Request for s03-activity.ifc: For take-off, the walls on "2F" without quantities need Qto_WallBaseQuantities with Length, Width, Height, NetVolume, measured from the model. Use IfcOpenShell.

First a look at what the model holds.

```python
import ifcopenshell
import ifcopenshell.util.element
import ifcopenshell.util.unit

model = ifcopenshell.open("s03-activity.ifc")
print(model.schema)
for unit_type in ("LENGTHUNIT", "AREAUNIT", "VOLUMEUNIT"):
    print(unit_type, ifcopenshell.util.unit.calculate_unit_scale(model, unit_type))
storey = next(s for s in model.by_type("IfcBuildingStorey") if s.Name == "2F")
walls = [e for e in ifcopenshell.util.element.get_decomposition(storey) if e.is_a("IfcWall")]
for e in sorted(walls, key=lambda e: e.id()):
    print(e.id(), e.is_a(), e.Name, list(ifcopenshell.util.element.get_psets(e, qtos_only=True)), sep=" | ")
```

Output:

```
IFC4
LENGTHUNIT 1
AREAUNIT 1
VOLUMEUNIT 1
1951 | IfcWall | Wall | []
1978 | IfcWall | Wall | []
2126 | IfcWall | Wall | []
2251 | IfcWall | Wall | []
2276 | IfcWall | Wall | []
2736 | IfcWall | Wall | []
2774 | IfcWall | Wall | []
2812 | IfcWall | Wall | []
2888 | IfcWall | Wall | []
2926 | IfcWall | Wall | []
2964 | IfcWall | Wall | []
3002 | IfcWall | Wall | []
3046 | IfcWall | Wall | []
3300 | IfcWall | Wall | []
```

```python
import ifcopenshell
import ifcopenshell.api.pset
import ifcopenshell.geom
import ifcopenshell.util.element
import ifcopenshell.util.shape
import ifcopenshell.util.unit

model = ifcopenshell.open("s03-activity.ifc")
unit_scale = ifcopenshell.util.unit.calculate_unit_scale(model)
volume_scale = ifcopenshell.util.unit.calculate_unit_scale(model, "VOLUMEUNIT")
settings = ifcopenshell.geom.settings()

storey = next(s for s in model.by_type("IfcBuildingStorey") if s.Name == "2F")
walls = [e for e in ifcopenshell.util.element.get_decomposition(storey) if e.is_a("IfcWall")]

for e in sorted(walls, key=lambda e: e.id()):
    if ifcopenshell.util.element.get_psets(e, qtos_only=True, should_inherit=False):
        continue
    # Geometry comes back in metres, in the element's own axes.
    shape = ifcopenshell.geom.create_shape(settings, e)
    values = {
        "Length": ifcopenshell.util.shape.get_x(shape.geometry) / unit_scale,
        "Width": ifcopenshell.util.shape.get_y(shape.geometry) / unit_scale,
        "Height": ifcopenshell.util.shape.get_z(shape.geometry) / unit_scale,
        "NetVolume": ifcopenshell.util.shape.get_volume(shape.geometry) / volume_scale,
    }
    qto = ifcopenshell.api.pset.add_qto(model, product=e, name="Qto_WallBaseQuantities")
    ifcopenshell.api.pset.edit_qto(model, qto=qto, properties=values)
    print(e.id(), {k: round(v, 3) for k, v in values.items()})

model.write("s03-activity_v2.ifc")
```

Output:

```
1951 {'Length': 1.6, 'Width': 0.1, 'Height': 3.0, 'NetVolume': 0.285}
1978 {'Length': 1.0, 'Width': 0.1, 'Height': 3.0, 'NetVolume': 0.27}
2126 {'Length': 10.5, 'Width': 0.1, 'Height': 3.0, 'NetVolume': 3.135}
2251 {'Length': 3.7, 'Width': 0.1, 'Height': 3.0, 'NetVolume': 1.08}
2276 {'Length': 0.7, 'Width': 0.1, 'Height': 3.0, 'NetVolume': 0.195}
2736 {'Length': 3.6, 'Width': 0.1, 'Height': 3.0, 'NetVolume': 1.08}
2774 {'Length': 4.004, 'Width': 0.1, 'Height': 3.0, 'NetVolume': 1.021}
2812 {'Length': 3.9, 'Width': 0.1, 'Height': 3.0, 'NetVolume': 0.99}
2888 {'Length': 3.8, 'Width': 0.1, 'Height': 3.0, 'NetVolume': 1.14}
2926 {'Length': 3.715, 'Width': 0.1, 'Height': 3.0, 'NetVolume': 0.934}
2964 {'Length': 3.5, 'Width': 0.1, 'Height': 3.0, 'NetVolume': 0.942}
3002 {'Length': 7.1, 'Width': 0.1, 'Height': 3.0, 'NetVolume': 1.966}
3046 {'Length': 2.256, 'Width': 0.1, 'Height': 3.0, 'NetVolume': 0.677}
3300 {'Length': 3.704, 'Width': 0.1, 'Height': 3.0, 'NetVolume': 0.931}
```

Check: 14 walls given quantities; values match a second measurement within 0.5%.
